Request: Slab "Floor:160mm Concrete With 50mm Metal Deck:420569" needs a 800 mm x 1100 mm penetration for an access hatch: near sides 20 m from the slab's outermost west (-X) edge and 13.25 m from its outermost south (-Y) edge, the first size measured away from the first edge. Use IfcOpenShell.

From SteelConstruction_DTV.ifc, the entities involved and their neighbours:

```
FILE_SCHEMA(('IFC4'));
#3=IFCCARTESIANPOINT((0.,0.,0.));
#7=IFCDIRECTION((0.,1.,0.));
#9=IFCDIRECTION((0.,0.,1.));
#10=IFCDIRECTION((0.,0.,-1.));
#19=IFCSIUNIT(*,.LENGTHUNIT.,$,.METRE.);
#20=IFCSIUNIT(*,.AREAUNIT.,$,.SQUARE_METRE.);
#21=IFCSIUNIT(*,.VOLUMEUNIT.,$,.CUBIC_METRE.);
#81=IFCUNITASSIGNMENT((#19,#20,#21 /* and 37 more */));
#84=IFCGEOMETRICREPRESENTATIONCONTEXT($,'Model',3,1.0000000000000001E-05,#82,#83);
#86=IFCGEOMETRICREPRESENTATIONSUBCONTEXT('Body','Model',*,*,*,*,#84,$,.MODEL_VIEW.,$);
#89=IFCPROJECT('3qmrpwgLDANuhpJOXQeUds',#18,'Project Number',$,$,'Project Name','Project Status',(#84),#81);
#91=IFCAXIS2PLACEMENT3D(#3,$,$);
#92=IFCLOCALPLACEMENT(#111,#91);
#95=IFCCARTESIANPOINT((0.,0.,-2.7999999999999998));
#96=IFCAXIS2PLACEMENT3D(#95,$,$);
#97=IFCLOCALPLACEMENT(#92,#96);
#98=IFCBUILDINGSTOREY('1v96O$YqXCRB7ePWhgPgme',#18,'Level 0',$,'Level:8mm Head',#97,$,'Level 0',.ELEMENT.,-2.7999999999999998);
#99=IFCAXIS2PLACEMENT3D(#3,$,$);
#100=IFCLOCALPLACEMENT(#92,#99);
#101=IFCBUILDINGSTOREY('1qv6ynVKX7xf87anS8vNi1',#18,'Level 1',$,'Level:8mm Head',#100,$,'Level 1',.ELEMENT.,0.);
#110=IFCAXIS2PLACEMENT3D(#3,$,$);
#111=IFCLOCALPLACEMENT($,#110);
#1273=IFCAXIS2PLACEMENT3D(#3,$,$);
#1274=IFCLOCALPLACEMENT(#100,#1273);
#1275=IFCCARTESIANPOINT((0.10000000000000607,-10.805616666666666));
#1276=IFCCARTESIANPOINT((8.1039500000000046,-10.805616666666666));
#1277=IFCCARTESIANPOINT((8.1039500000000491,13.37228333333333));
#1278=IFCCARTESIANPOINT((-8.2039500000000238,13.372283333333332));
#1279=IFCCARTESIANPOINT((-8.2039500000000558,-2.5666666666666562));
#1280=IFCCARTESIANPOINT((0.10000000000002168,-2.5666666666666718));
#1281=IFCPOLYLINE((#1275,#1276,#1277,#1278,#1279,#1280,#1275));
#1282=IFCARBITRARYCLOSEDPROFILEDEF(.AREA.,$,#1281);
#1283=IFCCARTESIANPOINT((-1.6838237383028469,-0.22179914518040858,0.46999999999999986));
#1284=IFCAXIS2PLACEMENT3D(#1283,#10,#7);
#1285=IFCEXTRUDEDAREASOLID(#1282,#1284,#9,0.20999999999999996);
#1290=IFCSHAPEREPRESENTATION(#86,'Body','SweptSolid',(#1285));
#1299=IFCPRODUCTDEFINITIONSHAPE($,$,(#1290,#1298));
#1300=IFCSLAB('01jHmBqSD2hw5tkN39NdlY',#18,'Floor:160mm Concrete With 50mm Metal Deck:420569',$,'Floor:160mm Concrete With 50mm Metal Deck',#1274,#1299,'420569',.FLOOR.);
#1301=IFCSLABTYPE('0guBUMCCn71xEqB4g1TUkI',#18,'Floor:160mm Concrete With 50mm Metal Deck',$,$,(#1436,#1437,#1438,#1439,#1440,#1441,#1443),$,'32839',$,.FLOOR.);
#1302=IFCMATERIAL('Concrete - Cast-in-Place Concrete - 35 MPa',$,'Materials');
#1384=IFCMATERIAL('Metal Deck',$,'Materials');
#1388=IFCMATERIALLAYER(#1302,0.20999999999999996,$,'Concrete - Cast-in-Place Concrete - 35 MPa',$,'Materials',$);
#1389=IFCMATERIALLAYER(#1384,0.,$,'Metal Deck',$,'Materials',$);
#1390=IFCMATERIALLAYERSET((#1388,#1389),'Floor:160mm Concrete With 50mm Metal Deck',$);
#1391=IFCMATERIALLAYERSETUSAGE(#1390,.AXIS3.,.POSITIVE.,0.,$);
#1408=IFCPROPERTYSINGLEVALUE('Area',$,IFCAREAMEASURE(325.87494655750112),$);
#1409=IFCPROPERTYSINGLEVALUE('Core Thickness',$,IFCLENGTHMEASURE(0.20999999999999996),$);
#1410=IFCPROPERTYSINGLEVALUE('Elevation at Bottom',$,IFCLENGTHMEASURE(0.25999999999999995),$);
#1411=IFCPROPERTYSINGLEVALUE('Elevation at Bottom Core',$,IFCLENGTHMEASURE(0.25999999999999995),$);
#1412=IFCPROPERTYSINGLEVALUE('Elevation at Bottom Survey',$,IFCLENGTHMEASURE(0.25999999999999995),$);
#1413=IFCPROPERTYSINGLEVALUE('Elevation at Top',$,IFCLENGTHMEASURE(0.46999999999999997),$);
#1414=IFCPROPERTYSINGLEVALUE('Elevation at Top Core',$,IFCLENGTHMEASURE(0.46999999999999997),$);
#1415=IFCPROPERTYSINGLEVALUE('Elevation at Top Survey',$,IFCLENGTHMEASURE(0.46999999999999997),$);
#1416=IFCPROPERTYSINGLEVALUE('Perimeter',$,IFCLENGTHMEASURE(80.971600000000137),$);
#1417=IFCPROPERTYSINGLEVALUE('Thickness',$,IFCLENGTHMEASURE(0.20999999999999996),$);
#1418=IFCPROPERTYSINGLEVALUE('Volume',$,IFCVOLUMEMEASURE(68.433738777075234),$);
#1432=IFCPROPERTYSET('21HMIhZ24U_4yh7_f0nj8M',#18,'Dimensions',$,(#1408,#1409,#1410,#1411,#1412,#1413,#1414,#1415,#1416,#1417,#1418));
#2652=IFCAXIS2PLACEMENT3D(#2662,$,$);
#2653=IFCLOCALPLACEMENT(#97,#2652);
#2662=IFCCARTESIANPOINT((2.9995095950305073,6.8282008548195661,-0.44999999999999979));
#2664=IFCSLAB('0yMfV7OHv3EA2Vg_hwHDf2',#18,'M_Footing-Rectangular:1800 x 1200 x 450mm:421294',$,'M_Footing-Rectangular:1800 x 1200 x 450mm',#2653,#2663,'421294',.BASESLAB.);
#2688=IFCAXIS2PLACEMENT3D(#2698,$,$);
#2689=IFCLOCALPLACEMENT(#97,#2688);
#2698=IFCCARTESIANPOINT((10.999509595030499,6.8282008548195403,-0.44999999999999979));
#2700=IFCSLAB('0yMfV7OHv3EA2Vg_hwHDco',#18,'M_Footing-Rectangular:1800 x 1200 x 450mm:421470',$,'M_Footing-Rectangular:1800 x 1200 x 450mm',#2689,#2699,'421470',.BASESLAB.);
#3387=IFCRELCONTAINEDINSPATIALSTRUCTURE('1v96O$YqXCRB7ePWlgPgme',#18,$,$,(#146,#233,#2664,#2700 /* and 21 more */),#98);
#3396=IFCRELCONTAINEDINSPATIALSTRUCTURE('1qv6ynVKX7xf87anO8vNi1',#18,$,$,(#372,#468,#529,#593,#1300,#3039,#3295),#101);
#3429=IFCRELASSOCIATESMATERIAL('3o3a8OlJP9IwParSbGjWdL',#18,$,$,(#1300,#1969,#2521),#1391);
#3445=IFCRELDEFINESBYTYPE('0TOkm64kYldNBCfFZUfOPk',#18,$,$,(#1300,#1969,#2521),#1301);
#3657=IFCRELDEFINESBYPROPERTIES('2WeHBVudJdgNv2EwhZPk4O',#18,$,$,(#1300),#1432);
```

```python
import numpy as np
import ifcopenshell
import ifcopenshell.api.feature
import ifcopenshell.api.geometry
import ifcopenshell.api.pset
import ifcopenshell.api.root
import ifcopenshell.geom
import ifcopenshell.util.element
import ifcopenshell.util.placement
import ifcopenshell.util.representation
import ifcopenshell.util.shape
import ifcopenshell.util.unit

model = ifcopenshell.open("SteelConstruction_DTV.ifc")
unit_scale = ifcopenshell.util.unit.calculate_unit_scale(model)
area_scale = ifcopenshell.util.unit.calculate_unit_scale(model, "AREAUNIT")
volume_scale = ifcopenshell.util.unit.calculate_unit_scale(model, "VOLUMEUNIT")
settings = ifcopenshell.geom.settings()


def volume(element):
    """Net volume in cubic metres, openings subtracted."""
    shape = ifcopenshell.geom.create_shape(settings, element)
    return ifcopenshell.util.shape.get_volume(shape.geometry)


slab = model.by_id(1300)
before = volume(slab)

# Extent in the slab's own axes, in metres. The edges named are its -X and -Y sides.
slab_shape = ifcopenshell.geom.create_shape(settings, slab)
vertices = ifcopenshell.util.shape.get_vertices(slab_shape.geometry)
x_min, y_min, bottom = vertices.min(axis=0)
top = vertices[:, 2].max()

opening = ifcopenshell.api.root.create_entity(model, ifc_class="IfcOpeningElement", name="Access hatch opening", predefined_type="OPENING")
context = ifcopenshell.util.representation.get_context(model, "Model", "Body", "MODEL_VIEW")
width, depth = 0.8, 1.1
outline = [(0.0, 0.0), (width, 0.0), (width, depth), (0.0, depth), (0.0, 0.0)]
# Overshoot both faces by 50 mm so the cut is clean.
shape = ifcopenshell.api.geometry.add_slab_representation(
    model, context=context, depth=top - bottom + 0.1, polyline=outline
)
ifcopenshell.api.geometry.assign_representation(model, product=opening, representation=shape)

matrix = ifcopenshell.util.placement.get_local_placement(slab.ObjectPlacement)
matrix[:, 3] = matrix @ np.append(np.array([x_min + 20, y_min + 13.25, bottom - 0.05]) / unit_scale, 1.0)
ifcopenshell.api.geometry.edit_object_placement(model, product=opening, matrix=matrix, is_si=False)
ifcopenshell.api.feature.add_feature(model, feature=opening, element=slab)

after = volume(slab)

# Update the slab's stored quantities.
pset = model.by_id(ifcopenshell.util.element.get_pset(slab, "Dimensions", should_inherit=False)["id"])
ifcopenshell.api.pset.edit_pset(model, pset=pset, properties={
    "Area": model.create_entity("IfcAreaMeasure", after / (top - bottom) / area_scale),
    "Volume": model.create_entity("IfcVolumeMeasure", after / volume_scale),
})

print(f"slab volume {before:.3f} -> {after:.3f} m3")

model.write("SteelConstruction_DTV-out.ifc")
```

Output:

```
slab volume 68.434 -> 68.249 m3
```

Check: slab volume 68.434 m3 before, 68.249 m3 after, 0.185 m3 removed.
